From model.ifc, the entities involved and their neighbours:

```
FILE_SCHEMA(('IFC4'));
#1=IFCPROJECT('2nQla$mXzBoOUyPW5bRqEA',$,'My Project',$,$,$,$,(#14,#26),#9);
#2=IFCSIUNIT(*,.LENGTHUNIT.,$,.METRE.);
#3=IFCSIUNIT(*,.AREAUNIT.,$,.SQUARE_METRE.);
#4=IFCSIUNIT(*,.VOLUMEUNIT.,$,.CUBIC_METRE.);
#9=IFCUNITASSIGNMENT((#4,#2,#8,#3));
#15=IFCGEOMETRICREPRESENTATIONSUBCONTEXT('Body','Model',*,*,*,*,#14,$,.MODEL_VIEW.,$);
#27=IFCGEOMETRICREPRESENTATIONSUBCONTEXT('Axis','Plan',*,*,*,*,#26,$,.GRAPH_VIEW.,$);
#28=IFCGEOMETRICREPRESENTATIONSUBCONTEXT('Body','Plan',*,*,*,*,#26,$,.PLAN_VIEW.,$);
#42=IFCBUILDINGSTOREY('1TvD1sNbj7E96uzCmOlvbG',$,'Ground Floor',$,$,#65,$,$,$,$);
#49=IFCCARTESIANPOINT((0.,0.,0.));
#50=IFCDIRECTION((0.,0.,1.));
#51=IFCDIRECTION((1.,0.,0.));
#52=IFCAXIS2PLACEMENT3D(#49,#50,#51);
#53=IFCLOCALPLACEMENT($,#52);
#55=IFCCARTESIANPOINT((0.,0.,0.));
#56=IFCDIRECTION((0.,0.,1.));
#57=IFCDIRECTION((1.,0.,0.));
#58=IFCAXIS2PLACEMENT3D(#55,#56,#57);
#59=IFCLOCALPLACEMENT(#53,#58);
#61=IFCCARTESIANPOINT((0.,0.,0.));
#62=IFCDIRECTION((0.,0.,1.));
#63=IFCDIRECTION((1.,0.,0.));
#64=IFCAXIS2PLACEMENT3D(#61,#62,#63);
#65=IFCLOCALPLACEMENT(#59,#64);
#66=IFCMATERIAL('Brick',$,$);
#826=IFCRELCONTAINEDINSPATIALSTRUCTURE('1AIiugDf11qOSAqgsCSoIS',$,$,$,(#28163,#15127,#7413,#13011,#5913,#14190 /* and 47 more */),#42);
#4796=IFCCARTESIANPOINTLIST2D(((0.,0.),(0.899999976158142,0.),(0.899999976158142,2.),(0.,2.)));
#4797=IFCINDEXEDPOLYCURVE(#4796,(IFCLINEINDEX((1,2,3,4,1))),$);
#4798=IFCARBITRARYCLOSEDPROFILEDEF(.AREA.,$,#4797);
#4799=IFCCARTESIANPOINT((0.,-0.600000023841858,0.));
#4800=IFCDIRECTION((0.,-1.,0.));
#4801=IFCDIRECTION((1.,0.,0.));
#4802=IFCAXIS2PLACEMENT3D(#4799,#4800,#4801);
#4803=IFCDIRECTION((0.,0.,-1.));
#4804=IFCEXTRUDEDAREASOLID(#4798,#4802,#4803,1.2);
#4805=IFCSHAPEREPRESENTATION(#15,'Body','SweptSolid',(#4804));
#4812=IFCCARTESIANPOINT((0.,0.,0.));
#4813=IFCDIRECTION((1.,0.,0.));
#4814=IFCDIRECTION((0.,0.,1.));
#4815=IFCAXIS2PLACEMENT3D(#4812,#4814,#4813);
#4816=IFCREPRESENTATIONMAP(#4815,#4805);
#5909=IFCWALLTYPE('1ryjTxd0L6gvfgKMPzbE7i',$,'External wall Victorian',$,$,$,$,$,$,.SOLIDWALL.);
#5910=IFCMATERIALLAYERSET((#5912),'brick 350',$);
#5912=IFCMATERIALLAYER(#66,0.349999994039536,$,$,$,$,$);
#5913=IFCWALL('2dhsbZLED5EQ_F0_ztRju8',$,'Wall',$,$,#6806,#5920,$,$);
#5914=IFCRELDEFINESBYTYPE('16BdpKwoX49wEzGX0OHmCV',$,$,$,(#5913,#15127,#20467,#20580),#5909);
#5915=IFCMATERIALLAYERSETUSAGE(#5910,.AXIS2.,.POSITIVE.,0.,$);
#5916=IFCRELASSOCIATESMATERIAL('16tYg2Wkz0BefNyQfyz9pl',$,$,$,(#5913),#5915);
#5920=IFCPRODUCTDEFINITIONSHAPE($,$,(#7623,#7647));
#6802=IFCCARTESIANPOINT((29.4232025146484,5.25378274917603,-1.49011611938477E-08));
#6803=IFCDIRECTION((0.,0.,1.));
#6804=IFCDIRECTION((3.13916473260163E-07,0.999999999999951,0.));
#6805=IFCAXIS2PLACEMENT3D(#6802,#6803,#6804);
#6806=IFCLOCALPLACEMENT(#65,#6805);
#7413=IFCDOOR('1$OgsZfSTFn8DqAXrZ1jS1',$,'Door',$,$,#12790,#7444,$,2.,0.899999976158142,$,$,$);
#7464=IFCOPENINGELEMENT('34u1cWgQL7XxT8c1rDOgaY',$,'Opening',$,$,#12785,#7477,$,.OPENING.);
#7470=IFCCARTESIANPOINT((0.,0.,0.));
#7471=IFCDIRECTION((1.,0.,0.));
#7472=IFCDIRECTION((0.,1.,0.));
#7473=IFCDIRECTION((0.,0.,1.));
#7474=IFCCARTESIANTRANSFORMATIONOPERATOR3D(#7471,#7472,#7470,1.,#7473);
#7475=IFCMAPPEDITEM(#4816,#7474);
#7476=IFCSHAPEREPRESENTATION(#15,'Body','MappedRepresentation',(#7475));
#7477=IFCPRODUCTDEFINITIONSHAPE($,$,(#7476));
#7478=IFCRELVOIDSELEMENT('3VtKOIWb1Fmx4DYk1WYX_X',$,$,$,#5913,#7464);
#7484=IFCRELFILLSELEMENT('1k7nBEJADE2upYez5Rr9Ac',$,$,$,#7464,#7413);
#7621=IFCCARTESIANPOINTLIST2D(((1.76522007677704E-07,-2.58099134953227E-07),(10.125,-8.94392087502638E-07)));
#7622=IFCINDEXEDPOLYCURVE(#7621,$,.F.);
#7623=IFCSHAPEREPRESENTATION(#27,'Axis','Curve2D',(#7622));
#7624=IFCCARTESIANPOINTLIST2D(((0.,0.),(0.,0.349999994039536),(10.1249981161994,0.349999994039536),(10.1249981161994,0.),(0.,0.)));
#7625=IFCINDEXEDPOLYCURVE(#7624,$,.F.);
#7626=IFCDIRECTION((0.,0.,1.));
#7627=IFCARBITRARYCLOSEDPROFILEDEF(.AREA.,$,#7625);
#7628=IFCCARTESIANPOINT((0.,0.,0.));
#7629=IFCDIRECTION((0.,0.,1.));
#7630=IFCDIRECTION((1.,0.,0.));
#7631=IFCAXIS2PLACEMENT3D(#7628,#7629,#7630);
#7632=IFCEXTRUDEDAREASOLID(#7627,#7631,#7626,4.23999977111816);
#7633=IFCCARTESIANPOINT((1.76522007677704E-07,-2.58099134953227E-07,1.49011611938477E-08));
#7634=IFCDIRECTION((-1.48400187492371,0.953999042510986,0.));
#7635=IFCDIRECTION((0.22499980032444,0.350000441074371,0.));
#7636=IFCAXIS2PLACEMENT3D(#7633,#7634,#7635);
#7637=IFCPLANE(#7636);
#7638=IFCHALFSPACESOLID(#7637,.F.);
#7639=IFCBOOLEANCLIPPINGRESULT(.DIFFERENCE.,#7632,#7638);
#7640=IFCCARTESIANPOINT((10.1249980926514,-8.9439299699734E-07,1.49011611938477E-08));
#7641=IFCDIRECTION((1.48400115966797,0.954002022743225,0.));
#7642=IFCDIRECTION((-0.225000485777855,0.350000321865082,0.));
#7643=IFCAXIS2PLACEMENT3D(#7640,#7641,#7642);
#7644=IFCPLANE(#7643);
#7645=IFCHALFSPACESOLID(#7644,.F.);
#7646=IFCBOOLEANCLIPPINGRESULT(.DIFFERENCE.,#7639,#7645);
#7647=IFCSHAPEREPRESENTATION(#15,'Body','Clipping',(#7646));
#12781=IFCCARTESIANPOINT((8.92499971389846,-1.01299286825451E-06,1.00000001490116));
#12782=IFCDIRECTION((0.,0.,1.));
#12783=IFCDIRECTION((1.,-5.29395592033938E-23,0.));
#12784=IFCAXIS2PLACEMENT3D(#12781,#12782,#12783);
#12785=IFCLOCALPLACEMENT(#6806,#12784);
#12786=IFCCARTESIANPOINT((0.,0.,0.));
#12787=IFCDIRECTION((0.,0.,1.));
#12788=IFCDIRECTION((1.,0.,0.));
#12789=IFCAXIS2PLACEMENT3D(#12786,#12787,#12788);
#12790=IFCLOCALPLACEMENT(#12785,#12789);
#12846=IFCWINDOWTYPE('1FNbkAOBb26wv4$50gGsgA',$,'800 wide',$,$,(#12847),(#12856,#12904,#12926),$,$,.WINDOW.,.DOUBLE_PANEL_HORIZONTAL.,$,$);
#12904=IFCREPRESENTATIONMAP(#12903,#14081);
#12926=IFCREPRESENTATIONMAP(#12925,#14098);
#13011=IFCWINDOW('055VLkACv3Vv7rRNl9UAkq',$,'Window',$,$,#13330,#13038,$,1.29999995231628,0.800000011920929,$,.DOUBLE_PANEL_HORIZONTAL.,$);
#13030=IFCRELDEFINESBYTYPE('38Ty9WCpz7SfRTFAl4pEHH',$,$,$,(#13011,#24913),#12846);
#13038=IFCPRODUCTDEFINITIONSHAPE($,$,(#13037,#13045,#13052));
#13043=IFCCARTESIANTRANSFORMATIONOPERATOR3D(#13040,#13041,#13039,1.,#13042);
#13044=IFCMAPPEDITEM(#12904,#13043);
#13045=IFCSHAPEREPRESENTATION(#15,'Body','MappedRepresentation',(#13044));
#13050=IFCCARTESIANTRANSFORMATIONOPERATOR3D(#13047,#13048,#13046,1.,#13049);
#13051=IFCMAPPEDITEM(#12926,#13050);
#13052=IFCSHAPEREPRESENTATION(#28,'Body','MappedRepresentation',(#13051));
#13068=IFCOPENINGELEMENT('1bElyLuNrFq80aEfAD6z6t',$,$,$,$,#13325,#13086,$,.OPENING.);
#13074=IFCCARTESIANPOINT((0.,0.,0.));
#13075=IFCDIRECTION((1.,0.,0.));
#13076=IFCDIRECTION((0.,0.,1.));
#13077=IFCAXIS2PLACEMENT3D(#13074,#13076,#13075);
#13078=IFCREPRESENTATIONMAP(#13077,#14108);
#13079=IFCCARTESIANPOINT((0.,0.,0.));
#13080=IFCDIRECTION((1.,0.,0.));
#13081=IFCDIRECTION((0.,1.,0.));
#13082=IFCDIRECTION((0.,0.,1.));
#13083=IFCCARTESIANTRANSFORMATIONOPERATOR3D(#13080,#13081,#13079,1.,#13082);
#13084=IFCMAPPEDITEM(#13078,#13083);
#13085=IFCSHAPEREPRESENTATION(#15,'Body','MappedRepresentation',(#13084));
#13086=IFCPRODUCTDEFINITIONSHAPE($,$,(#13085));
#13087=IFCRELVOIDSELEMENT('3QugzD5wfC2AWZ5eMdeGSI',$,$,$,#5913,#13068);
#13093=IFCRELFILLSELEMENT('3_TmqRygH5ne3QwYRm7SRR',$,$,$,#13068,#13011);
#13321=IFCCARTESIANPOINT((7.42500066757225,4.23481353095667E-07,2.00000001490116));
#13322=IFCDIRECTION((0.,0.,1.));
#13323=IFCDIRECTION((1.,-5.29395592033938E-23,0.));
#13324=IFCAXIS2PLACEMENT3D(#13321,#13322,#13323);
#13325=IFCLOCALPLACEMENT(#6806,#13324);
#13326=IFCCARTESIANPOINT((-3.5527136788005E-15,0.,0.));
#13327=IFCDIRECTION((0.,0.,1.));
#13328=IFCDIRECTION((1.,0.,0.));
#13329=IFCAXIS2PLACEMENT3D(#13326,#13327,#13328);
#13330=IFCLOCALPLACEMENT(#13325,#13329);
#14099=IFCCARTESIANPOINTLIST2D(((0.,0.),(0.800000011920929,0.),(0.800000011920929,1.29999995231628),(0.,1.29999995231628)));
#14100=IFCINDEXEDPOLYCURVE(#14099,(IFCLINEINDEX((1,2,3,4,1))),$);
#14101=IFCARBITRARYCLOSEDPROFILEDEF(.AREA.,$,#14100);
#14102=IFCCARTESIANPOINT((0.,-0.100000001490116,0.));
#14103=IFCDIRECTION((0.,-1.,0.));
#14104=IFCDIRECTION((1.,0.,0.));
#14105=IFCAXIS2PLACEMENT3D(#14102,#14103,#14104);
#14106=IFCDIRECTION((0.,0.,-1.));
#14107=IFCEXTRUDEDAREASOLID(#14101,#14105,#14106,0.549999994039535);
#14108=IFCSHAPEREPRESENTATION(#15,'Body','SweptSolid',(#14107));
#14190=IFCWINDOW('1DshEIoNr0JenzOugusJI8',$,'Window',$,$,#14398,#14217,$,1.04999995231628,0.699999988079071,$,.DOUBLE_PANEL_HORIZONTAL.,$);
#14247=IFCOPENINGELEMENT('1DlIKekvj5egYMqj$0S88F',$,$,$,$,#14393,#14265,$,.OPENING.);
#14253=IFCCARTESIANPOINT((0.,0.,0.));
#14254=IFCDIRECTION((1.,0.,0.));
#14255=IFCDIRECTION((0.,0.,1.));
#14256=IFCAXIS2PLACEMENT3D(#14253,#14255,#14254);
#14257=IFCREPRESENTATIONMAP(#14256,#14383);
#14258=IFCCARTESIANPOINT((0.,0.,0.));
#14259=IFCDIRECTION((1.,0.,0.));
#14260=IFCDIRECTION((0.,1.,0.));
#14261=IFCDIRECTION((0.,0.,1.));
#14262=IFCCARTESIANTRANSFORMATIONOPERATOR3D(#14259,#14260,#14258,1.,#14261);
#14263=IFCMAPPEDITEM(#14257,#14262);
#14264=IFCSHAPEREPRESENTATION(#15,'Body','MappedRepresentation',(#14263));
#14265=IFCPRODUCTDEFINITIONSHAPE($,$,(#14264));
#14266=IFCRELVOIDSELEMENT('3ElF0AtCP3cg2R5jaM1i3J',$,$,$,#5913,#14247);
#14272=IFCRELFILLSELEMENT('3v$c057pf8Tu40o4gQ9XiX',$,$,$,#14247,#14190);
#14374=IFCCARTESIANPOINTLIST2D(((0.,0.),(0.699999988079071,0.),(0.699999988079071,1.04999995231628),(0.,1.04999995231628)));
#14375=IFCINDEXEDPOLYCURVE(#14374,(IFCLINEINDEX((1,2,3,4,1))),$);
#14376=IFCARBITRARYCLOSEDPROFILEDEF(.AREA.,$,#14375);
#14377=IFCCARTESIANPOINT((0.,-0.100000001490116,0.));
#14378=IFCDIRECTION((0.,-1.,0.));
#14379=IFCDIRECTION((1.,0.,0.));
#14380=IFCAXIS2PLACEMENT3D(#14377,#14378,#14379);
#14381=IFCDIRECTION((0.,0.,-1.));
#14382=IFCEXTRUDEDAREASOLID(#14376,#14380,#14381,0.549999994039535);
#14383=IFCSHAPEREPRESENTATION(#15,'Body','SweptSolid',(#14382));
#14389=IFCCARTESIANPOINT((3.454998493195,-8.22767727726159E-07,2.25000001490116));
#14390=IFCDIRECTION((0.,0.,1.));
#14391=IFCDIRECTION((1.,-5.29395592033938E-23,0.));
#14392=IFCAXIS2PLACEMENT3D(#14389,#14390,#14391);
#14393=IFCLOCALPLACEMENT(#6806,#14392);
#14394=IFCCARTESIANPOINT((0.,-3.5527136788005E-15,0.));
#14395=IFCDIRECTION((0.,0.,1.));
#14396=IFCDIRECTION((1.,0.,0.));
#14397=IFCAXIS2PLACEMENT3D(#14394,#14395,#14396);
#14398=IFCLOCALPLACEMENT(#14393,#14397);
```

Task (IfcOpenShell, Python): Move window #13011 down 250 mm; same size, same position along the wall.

```python
import numpy as np
import ifcopenshell
import ifcopenshell.api.geometry
import ifcopenshell.util.placement
import ifcopenshell.util.unit

model = ifcopenshell.open("model.ifc")
unit_scale = ifcopenshell.util.unit.calculate_unit_scale(model)

window = model.by_id(13011)
opening = window.FillsVoids[0].RelatingOpeningElement
dz = -0.25

shift = np.array([0.0, 0.0, dz])
# The window is placed relative to its opening, so it follows when the opening moves.
matrix = ifcopenshell.util.placement.get_local_placement(opening.ObjectPlacement)
matrix[:3, 3] += shift
ifcopenshell.api.geometry.edit_object_placement(
    model, product=opening, matrix=matrix, is_si=False, should_transform_children=True
)

print(f"moved by {dz * unit_scale:+.3f} m")

model.write("model-out.ifc")
```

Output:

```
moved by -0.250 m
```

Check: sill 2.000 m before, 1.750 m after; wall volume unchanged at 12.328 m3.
